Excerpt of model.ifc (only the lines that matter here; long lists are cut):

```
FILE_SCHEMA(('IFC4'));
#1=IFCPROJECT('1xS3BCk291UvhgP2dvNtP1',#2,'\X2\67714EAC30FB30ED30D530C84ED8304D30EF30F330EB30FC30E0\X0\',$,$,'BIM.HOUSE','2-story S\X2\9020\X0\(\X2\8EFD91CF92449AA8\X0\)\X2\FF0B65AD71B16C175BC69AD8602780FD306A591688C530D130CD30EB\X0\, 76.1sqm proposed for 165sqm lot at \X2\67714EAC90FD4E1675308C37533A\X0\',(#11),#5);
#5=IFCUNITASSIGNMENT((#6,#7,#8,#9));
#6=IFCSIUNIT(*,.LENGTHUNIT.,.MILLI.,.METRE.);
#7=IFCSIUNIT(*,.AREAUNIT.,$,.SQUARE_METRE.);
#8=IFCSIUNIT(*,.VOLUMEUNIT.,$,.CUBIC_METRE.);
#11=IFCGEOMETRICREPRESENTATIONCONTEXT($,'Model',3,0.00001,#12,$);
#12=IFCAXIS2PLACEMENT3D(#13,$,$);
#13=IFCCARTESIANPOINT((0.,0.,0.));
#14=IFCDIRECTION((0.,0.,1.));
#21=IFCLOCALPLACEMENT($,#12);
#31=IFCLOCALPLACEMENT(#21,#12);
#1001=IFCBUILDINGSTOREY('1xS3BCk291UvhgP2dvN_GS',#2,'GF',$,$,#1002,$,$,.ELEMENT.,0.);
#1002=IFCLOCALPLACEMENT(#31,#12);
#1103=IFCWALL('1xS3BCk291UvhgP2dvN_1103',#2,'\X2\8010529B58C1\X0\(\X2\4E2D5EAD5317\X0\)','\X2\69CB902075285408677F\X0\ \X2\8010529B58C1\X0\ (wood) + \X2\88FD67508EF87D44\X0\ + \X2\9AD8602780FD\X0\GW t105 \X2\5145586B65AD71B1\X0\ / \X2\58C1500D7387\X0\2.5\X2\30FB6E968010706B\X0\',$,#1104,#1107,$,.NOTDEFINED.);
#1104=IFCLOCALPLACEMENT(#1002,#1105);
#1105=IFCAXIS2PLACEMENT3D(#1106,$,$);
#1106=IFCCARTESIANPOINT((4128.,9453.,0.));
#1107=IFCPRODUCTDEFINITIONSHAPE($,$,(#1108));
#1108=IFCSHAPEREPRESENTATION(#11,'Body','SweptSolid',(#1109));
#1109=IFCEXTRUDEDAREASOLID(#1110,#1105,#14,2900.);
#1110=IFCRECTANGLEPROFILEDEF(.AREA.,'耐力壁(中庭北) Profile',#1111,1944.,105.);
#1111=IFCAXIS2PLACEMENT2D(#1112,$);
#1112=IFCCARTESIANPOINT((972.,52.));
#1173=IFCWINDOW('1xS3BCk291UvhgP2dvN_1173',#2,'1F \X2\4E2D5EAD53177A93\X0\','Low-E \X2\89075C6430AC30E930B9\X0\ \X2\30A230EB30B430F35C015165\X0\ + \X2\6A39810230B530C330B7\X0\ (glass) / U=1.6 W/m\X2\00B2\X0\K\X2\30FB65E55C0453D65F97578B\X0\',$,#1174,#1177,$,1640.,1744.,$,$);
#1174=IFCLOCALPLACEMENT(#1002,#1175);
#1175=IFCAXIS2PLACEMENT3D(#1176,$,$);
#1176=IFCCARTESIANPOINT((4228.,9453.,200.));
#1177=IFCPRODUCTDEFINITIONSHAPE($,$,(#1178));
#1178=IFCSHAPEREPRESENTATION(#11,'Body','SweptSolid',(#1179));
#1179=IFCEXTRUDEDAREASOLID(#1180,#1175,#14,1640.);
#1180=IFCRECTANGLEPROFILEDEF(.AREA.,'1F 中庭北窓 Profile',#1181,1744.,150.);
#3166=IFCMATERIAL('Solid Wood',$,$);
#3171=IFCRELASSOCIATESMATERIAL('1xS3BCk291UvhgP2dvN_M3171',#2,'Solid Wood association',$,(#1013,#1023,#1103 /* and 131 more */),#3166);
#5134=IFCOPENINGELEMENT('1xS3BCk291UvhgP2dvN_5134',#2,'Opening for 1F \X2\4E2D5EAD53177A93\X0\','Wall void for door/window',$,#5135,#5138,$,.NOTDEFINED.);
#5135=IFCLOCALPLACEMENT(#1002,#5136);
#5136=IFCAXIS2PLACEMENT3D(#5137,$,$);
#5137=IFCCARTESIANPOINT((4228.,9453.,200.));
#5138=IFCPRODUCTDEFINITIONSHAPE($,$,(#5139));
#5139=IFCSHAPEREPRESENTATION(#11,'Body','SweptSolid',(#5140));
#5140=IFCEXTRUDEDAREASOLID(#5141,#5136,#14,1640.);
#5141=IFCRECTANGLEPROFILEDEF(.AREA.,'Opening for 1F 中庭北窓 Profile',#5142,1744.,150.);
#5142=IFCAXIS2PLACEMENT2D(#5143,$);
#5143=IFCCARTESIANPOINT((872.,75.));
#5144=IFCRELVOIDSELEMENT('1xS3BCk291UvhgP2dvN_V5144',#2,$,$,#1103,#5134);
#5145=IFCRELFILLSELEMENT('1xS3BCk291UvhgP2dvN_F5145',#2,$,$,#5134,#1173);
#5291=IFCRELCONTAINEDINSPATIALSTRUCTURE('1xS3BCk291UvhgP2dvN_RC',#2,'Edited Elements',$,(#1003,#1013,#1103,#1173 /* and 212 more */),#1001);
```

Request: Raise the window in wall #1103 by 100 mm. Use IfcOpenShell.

```python
import numpy as np
import ifcopenshell
import ifcopenshell.api.geometry
import ifcopenshell.util.placement
import ifcopenshell.util.unit

model = ifcopenshell.open("model.ifc")
unit_scale = ifcopenshell.util.unit.calculate_unit_scale(model)

window = model.by_guid("1xS3BCk291UvhgP2dvN_1173")
opening = window.FillsVoids[0].RelatingOpeningElement
dz = 100.0

shift = np.array([0.0, 0.0, dz])
# The window is not placed relative to its opening, so move both.
for product in (opening, window):
    matrix = ifcopenshell.util.placement.get_local_placement(product.ObjectPlacement)
    matrix[:3, 3] += shift
    ifcopenshell.api.geometry.edit_object_placement(model, product=product, matrix=matrix, is_si=False)

print(f"moved by {dz * unit_scale:+.3f} m")

model.write("model_v2.ifc")
```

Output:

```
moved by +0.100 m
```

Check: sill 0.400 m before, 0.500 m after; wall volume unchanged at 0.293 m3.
